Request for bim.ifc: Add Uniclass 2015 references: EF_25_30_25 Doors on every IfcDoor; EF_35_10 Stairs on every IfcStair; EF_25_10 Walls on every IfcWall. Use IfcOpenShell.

First a look at what the model holds.

```python
import ifcopenshell

model = ifcopenshell.open("bim.ifc")
print(model.schema)
print("classifications:", [c.Name for c in model.by_type("IfcClassification")])
for ifc_class in ("IfcDoor", "IfcRoof", "IfcStair", "IfcWall", "IfcWindow"):
    print(ifc_class, len(model.by_type(ifc_class)))
```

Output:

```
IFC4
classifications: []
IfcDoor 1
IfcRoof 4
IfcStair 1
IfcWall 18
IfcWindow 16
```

```python
import ifcopenshell
import ifcopenshell.api.classification

model = ifcopenshell.open("bim.ifc")

system = ifcopenshell.api.classification.add_classification(model, classification="Uniclass 2015")

codes = {
    "IfcDoor": ("EF_25_30_25", "Doors"),
    "IfcStair": ("EF_35_10", "Stairs"),
    "IfcWall": ("EF_25_10", "Walls"),
}
for ifc_class, (code, name) in codes.items():
    products = model.by_type(ifc_class)
    ifcopenshell.api.classification.add_reference(
        model, products=products, classification=system, identification=code, name=name
    )
    print(code, len(products))

model.write("bim-out.ifc")
```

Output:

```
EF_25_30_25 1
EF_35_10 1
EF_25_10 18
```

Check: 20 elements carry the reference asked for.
